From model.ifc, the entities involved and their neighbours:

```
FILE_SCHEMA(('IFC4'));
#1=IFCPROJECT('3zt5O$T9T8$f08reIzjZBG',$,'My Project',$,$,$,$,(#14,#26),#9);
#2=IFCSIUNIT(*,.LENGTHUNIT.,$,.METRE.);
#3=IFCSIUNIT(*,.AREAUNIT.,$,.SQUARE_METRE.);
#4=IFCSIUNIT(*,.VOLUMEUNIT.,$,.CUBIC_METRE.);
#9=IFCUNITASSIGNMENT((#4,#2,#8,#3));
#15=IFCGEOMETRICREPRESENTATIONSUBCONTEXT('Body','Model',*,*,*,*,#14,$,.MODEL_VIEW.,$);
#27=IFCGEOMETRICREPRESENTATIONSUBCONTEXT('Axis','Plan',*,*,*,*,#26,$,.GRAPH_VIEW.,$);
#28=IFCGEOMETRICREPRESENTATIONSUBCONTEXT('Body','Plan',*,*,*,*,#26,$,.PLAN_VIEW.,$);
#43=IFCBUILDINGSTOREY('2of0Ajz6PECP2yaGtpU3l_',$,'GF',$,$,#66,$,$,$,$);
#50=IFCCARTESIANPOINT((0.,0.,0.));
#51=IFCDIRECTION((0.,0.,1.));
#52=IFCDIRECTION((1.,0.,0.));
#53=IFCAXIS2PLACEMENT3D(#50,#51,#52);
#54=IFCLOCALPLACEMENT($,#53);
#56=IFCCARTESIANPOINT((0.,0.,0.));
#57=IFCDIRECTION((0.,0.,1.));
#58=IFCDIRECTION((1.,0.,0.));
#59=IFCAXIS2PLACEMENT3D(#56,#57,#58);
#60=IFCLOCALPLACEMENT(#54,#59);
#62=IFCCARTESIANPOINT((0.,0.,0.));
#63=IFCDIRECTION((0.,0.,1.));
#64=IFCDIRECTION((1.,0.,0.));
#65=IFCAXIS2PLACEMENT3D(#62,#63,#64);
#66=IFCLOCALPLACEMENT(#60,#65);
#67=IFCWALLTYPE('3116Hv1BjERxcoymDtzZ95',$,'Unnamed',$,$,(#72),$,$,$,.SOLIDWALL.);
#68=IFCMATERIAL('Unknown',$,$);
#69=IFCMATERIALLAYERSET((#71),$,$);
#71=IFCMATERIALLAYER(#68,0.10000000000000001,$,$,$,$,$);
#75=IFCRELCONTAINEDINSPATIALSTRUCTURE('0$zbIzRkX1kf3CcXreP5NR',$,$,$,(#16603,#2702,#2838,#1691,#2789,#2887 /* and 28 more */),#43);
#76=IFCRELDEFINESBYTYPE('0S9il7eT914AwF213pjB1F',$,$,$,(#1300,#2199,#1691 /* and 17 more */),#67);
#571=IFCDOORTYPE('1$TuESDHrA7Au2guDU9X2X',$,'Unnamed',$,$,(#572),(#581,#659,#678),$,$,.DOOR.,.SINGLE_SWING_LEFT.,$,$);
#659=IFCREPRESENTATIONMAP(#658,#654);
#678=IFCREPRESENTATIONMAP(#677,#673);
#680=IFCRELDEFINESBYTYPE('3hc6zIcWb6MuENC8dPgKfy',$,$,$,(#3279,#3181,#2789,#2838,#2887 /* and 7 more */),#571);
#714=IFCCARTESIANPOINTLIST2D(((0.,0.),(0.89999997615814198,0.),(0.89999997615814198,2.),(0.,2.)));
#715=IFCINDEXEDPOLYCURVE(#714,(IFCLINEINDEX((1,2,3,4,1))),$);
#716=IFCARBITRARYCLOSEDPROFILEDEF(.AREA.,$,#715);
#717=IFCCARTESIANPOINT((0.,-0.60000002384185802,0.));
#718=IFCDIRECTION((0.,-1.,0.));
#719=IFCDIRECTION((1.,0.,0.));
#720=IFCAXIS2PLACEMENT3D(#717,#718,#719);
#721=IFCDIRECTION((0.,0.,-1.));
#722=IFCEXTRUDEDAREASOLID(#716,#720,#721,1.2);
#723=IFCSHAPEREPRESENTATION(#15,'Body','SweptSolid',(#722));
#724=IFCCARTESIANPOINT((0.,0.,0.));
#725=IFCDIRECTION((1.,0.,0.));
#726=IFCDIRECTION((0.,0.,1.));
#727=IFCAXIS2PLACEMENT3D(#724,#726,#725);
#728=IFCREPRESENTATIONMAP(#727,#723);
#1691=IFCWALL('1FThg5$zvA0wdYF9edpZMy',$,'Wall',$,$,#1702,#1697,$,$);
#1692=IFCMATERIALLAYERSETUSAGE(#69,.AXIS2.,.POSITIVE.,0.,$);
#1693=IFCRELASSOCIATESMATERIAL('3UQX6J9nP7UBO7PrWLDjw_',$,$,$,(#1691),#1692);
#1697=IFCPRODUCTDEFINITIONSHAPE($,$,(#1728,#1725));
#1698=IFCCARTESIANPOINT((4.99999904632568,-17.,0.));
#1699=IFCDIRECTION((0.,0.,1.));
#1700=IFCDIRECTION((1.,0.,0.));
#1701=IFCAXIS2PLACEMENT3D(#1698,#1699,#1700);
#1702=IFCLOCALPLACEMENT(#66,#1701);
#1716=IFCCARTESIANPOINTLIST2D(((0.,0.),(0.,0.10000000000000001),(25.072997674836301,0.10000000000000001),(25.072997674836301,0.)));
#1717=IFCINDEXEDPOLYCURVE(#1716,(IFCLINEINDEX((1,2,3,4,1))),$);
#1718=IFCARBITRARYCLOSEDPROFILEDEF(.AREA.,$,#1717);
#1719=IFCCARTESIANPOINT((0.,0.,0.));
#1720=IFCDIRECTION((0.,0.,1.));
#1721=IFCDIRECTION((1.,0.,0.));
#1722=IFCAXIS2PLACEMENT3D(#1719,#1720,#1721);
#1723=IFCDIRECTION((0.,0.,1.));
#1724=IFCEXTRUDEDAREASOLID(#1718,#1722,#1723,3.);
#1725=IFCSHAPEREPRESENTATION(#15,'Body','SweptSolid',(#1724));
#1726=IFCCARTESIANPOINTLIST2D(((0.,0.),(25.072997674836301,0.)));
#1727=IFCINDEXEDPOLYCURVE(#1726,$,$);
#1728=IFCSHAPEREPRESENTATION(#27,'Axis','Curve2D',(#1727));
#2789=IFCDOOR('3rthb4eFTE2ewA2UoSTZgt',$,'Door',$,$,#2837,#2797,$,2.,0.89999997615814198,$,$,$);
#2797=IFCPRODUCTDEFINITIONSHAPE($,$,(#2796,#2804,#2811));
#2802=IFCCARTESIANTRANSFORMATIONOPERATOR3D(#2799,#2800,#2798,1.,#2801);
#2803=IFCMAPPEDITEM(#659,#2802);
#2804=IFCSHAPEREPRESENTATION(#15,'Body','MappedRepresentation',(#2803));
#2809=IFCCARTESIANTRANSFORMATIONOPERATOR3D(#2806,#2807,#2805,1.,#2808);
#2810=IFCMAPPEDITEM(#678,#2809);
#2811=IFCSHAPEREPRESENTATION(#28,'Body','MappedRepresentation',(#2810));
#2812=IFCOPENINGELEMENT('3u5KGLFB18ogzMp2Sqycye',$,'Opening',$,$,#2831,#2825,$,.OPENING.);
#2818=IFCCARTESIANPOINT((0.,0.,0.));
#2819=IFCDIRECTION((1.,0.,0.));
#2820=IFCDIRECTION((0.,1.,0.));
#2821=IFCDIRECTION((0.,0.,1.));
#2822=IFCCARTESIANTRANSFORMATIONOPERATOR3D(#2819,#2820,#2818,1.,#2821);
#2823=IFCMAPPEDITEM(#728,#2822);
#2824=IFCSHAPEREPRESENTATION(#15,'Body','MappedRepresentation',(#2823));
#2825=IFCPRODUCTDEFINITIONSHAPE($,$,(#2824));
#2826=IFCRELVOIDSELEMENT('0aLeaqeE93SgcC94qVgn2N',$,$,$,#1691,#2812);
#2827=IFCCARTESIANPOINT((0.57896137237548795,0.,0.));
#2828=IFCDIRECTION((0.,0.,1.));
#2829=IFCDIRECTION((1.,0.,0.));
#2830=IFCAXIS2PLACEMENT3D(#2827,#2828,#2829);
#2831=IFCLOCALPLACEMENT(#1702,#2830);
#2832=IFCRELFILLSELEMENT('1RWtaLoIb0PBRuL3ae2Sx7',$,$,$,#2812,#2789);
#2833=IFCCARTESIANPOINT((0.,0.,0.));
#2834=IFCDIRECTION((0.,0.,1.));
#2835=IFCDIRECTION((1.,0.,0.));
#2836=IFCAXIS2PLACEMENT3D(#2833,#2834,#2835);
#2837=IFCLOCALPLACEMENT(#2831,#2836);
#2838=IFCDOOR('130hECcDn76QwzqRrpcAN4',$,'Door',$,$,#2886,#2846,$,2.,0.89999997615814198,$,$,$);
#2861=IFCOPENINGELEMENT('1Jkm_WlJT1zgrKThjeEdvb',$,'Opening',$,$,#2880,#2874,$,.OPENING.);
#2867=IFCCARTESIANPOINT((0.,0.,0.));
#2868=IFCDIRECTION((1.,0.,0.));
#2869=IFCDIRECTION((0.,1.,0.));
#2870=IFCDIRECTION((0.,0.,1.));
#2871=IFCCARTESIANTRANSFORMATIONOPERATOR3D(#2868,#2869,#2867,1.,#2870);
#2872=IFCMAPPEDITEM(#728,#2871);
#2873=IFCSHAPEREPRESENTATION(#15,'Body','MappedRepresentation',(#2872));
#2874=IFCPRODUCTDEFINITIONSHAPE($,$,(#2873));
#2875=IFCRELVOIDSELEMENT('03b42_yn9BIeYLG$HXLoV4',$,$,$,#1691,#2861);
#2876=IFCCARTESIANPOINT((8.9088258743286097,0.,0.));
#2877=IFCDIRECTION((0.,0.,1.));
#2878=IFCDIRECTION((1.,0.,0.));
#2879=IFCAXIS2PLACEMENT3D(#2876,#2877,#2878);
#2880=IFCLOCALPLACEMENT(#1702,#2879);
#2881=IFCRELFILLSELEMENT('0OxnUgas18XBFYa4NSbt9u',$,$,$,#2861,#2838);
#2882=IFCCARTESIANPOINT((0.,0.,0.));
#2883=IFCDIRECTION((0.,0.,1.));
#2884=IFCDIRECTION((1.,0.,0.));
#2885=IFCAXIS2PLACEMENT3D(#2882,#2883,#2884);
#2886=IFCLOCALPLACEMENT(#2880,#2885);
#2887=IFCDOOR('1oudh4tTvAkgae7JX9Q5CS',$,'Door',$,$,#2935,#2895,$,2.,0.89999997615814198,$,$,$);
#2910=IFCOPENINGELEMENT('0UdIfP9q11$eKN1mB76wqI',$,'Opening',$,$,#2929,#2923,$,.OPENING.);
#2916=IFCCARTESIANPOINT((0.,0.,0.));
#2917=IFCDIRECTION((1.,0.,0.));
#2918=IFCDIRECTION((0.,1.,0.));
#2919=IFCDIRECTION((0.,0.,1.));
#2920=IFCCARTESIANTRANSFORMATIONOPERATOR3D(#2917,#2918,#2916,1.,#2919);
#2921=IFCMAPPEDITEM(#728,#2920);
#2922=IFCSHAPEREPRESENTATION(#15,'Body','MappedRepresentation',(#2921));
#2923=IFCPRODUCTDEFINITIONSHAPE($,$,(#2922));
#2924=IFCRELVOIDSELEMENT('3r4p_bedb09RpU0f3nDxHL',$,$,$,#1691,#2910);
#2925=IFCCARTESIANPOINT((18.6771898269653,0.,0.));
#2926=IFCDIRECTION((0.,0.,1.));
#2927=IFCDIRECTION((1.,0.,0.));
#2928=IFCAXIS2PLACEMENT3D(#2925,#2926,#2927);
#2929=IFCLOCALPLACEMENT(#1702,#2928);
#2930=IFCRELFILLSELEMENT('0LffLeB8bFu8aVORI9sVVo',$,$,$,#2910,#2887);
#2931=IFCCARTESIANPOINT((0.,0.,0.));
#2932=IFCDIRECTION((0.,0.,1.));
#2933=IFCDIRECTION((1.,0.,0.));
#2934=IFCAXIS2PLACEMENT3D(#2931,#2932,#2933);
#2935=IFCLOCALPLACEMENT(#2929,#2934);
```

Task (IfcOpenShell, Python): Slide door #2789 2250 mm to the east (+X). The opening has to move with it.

```python
import ifcopenshell
import ifcopenshell.api.geometry
import ifcopenshell.util.placement

model = ifcopenshell.open("model.ifc")

door = model.by_guid("3rthb4eFTE2ewA2UoSTZgt")
opening = door.FillsVoids[0].RelatingOpeningElement
wall = opening.VoidsElements[0].RelatingBuildingElement

wall_matrix = ifcopenshell.util.placement.get_local_placement(wall.ObjectPlacement)
shift = wall_matrix[:3, 0] * 2.25
before = ifcopenshell.util.placement.get_local_placement(door.ObjectPlacement)[:3, 3].copy()

# The door is placed relative to its opening, so it follows when the opening moves.
matrix = ifcopenshell.util.placement.get_local_placement(opening.ObjectPlacement)
matrix[:3, 3] += shift
ifcopenshell.api.geometry.edit_object_placement(
    model, product=opening, matrix=matrix, is_si=False, should_transform_children=True
)

after = ifcopenshell.util.placement.get_local_placement(door.ObjectPlacement)[:3, 3]
print("door moved by", (after - before).round(3) + 0.0)

model.write("model-out.ifc")
```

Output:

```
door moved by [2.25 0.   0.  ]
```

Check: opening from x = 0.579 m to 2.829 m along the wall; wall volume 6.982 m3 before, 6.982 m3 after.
